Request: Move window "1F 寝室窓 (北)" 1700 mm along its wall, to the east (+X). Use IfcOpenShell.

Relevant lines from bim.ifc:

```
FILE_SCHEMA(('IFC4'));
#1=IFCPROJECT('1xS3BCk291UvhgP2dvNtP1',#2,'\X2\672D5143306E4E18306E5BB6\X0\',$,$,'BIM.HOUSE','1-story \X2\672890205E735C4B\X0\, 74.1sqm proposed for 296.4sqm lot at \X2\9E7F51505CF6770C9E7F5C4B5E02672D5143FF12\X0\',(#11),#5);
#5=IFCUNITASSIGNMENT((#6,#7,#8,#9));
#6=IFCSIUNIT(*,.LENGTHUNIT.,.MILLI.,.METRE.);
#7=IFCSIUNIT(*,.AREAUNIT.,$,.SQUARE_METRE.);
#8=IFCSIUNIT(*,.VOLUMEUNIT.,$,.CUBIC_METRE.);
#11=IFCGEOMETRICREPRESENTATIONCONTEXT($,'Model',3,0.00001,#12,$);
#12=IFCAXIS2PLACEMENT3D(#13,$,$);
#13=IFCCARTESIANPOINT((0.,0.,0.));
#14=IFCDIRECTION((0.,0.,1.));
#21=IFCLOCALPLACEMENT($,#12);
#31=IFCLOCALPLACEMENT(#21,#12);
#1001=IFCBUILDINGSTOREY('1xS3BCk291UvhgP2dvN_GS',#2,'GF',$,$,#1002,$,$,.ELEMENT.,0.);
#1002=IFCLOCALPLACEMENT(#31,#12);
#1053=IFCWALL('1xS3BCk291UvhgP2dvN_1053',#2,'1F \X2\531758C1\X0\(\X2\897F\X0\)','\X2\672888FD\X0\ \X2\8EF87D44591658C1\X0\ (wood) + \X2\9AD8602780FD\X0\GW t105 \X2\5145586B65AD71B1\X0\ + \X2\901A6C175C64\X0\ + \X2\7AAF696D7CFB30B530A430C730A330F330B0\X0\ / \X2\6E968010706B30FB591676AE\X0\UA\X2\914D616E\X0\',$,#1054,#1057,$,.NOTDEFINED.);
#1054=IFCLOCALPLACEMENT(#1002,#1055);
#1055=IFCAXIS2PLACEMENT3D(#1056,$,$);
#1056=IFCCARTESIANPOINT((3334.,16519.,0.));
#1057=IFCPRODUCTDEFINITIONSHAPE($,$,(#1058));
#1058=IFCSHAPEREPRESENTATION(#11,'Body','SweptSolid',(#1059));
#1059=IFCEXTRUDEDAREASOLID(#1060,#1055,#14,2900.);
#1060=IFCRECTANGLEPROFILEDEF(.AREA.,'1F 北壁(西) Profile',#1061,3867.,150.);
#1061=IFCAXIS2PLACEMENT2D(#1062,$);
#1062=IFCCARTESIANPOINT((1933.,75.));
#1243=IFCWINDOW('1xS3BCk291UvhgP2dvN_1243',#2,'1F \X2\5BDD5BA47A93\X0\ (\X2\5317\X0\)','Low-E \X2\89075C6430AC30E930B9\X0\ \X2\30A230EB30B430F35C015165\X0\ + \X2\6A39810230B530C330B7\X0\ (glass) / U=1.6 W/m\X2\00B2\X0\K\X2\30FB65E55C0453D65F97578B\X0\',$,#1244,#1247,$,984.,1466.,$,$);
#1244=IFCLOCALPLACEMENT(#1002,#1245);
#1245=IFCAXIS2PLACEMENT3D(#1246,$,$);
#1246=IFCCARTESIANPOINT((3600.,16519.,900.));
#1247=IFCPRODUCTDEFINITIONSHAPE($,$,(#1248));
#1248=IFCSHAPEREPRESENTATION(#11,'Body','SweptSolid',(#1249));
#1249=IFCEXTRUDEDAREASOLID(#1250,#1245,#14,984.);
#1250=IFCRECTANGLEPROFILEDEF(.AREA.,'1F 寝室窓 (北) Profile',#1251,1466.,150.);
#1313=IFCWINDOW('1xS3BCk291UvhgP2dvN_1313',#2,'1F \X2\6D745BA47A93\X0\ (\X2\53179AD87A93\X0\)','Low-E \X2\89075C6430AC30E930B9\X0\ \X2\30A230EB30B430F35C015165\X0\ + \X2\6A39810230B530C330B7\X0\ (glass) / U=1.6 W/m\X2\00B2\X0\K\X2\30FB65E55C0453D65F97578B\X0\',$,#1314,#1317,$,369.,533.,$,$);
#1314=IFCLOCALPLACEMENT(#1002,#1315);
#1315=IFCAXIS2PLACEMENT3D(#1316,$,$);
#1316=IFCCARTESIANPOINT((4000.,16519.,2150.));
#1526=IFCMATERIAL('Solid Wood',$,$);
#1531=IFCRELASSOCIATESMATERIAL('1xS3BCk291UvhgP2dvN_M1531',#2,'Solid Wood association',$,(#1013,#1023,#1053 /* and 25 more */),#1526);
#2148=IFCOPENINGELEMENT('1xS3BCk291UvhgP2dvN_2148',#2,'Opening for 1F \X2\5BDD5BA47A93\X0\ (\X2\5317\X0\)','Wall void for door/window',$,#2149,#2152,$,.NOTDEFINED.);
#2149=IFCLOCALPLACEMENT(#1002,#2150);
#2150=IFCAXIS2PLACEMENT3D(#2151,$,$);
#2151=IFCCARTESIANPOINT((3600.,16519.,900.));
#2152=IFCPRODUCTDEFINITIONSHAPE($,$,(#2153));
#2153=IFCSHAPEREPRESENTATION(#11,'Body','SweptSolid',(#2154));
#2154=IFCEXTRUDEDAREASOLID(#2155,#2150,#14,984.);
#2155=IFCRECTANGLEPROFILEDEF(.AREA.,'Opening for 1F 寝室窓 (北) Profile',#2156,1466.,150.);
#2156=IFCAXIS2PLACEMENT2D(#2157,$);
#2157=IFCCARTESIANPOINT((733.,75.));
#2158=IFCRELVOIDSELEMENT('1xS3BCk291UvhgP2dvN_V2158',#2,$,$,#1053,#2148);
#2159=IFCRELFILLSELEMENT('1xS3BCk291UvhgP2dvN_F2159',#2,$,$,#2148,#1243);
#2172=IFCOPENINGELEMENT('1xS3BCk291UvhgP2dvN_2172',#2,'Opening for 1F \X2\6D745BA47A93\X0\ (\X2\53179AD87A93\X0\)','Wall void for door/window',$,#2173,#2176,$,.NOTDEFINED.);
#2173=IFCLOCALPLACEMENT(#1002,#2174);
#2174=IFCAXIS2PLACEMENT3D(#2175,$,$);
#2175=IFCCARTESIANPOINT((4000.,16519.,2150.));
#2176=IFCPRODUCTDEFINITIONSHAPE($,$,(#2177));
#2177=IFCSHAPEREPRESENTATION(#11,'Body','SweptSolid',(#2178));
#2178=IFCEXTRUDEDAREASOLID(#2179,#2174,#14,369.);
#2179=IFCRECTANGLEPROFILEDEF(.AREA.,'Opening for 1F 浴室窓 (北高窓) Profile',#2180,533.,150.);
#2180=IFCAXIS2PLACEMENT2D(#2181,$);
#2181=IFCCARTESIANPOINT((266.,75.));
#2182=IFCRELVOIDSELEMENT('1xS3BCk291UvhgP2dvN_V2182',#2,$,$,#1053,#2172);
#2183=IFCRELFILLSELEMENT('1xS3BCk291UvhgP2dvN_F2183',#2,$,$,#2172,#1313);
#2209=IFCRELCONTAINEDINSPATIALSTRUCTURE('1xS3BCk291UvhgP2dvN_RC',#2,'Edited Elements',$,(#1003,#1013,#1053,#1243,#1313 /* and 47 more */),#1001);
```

```python
import ifcopenshell
import ifcopenshell.api.geometry
import ifcopenshell.util.placement

model = ifcopenshell.open("bim.ifc")

window = model.by_guid("1xS3BCk291UvhgP2dvN_1243")
opening = window.FillsVoids[0].RelatingOpeningElement
wall = opening.VoidsElements[0].RelatingBuildingElement

wall_matrix = ifcopenshell.util.placement.get_local_placement(wall.ObjectPlacement)
shift = wall_matrix[:3, 0] * 1700.0
before = ifcopenshell.util.placement.get_local_placement(window.ObjectPlacement)[:3, 3].copy()

# The window is not placed relative to its opening, so move both.
for product in (opening, window):
    matrix = ifcopenshell.util.placement.get_local_placement(product.ObjectPlacement)
    matrix[:3, 3] += shift
    ifcopenshell.api.geometry.edit_object_placement(model, product=product, matrix=matrix, is_si=False)

after = ifcopenshell.util.placement.get_local_placement(window.ObjectPlacement)[:3, 3]
print("window moved by", (after - before).round(3) + 0.0)

model.write("bim_v2.ifc")
```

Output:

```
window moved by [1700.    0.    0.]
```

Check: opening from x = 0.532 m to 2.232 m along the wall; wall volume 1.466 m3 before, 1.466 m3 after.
